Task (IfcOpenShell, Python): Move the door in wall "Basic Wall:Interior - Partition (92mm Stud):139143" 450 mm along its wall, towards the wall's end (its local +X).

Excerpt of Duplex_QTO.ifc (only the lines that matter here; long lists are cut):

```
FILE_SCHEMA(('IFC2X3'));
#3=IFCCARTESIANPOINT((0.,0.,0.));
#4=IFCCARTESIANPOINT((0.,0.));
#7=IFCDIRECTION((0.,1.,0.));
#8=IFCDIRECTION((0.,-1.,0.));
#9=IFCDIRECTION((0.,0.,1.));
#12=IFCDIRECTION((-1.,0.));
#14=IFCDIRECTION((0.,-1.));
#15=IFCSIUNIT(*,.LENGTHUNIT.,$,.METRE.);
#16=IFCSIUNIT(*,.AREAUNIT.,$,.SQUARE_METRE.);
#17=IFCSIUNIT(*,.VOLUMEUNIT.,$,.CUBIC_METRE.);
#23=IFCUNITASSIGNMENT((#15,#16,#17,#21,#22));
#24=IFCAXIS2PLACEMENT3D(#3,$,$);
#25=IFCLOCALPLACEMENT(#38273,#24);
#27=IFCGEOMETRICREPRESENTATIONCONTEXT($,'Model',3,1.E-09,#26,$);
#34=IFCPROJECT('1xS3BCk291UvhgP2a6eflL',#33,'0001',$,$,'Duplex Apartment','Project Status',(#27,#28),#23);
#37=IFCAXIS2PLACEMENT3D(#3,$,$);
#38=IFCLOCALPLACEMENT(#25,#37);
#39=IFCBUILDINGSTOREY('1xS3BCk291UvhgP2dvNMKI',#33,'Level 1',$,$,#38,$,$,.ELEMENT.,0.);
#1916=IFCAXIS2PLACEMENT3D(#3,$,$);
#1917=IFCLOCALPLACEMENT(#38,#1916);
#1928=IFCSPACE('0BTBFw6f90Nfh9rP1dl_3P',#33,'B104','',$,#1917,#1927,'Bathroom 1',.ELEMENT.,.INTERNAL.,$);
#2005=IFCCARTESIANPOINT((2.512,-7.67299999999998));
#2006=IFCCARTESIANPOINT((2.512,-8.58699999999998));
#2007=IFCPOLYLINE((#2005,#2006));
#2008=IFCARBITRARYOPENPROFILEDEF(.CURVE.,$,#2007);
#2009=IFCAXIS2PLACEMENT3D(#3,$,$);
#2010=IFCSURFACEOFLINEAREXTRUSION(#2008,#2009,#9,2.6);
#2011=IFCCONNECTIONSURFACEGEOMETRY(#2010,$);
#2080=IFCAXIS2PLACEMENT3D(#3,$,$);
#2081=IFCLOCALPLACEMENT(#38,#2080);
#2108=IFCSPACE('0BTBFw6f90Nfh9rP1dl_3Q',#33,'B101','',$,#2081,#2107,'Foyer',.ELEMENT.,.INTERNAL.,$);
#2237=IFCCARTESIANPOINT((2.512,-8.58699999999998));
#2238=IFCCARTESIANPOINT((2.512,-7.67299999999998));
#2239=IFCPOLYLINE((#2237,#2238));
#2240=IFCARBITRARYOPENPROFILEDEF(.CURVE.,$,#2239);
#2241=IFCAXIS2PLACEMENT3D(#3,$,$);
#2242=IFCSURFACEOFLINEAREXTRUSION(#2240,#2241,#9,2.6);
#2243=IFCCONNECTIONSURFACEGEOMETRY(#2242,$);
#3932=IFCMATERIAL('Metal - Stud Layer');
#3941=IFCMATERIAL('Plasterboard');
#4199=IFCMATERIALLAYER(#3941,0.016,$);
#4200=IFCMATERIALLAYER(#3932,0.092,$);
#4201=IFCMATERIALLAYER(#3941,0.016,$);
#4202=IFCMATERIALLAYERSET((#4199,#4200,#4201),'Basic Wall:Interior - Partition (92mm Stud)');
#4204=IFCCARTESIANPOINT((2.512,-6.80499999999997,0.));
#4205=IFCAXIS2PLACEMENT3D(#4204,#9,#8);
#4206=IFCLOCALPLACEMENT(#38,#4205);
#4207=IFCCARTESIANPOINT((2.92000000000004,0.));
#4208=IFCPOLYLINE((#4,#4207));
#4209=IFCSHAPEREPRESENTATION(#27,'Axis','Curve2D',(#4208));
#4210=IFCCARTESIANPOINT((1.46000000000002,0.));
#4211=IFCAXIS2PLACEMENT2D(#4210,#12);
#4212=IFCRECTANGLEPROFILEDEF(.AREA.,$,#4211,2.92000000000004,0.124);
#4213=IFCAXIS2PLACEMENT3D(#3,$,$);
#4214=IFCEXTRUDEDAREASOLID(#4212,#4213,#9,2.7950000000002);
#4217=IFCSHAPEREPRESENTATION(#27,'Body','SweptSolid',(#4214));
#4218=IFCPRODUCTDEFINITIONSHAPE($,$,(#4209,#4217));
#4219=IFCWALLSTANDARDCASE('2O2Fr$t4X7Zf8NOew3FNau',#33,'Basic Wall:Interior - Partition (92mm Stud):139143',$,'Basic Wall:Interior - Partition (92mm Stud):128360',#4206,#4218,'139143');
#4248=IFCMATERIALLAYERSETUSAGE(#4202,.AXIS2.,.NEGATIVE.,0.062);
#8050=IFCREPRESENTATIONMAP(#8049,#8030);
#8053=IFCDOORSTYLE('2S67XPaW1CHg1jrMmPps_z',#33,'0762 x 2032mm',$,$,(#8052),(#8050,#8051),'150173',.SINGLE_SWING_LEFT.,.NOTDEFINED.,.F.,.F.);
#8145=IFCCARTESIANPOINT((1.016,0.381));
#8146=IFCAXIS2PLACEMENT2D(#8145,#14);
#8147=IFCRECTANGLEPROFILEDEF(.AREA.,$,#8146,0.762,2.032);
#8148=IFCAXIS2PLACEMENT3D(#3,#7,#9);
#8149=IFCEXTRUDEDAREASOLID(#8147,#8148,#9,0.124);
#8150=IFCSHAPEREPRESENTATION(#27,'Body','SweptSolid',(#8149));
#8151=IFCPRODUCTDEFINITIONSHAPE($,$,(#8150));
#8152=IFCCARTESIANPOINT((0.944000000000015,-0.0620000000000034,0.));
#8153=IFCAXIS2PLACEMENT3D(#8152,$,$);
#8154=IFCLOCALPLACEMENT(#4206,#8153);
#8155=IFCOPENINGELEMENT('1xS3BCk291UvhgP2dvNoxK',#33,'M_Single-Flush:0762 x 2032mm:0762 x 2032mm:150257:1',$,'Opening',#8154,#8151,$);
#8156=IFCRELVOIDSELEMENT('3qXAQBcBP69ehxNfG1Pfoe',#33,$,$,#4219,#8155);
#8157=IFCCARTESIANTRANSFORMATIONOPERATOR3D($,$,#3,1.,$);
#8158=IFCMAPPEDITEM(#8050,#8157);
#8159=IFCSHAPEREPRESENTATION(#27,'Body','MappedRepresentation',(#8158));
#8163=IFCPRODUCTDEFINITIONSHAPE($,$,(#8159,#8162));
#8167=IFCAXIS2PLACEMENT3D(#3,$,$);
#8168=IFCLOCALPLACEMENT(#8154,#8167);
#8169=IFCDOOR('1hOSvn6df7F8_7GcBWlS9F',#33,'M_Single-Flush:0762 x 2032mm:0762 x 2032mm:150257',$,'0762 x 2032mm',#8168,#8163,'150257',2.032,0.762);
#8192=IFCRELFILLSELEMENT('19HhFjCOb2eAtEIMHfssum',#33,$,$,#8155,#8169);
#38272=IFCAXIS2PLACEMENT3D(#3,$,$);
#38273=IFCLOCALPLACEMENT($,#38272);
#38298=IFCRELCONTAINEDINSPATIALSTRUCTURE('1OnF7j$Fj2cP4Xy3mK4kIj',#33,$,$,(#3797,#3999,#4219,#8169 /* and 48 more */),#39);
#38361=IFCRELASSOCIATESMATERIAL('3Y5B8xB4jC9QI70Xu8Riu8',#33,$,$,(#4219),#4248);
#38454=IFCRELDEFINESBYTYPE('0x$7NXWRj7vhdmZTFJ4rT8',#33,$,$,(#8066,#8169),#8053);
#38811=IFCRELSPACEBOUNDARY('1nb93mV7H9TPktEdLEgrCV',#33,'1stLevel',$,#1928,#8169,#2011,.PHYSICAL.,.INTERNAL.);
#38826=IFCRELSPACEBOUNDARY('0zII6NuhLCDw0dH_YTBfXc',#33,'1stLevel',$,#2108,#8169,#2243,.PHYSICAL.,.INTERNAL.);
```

```python
import numpy as np
import ifcopenshell
import ifcopenshell.api.geometry
import ifcopenshell.util.placement

model = ifcopenshell.open("Duplex_QTO.ifc")

door = model.by_guid("1hOSvn6df7F8_7GcBWlS9F")
opening = door.FillsVoids[0].RelatingOpeningElement
wall = opening.VoidsElements[0].RelatingBuildingElement

wall_matrix = ifcopenshell.util.placement.get_local_placement(wall.ObjectPlacement)
shift = wall_matrix[:3, 0] * 0.45
before = ifcopenshell.util.placement.get_local_placement(door.ObjectPlacement)[:3, 3].copy()

# The door is placed relative to its opening, so it follows when the opening moves.
matrix = ifcopenshell.util.placement.get_local_placement(opening.ObjectPlacement)
matrix[:3, 3] += shift
ifcopenshell.api.geometry.edit_object_placement(
    model, product=opening, matrix=matrix, is_si=False, should_transform_children=True
)

# Space boundary surfaces are stored in each space's coordinates; move them too.
for rel in door.ProvidesBoundaries:
    if not rel.ConnectionGeometry:
        continue
    surface = rel.ConnectionGeometry.SurfaceOnRelatingElement
    space_matrix = ifcopenshell.util.placement.get_local_placement(rel.RelatingSpace.ObjectPlacement)
    point = np.array(surface.Position.Location.Coordinates) + space_matrix[:3, :3].T @ shift
    surface.Position = model.createIfcAxis2Placement3D(
        model.createIfcCartesianPoint(point.tolist()), surface.Position.Axis, surface.Position.RefDirection
    )

after = ifcopenshell.util.placement.get_local_placement(door.ObjectPlacement)[:3, 3]
print("door moved by", (after - before).round(3) + 0.0)

model.write("Duplex_QTO_edited.ifc")
```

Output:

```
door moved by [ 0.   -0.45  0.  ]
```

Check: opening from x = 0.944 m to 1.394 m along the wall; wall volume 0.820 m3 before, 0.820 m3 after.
